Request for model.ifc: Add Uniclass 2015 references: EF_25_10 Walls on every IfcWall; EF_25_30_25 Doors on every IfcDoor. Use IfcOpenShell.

First a look at what the model holds.

```python
import ifcopenshell

model = ifcopenshell.open("model.ifc")
print(model.schema)
print("classifications:", [c.Name for c in model.by_type("IfcClassification")])
for ifc_class in ("IfcDoor", "IfcRoof", "IfcStair", "IfcWall", "IfcWindow"):
    print(ifc_class, len(model.by_type(ifc_class)))
```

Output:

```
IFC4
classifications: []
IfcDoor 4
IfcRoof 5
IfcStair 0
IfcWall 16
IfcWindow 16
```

```python
import ifcopenshell
import ifcopenshell.api.classification

model = ifcopenshell.open("model.ifc")

system = ifcopenshell.api.classification.add_classification(model, classification="Uniclass 2015")

codes = {
    "IfcWall": ("EF_25_10", "Walls"),
    "IfcDoor": ("EF_25_30_25", "Doors"),
}
for ifc_class, (code, name) in codes.items():
    products = model.by_type(ifc_class)
    ifcopenshell.api.classification.add_reference(
        model, products=products, classification=system, identification=code, name=name
    )
    print(code, len(products))

model.write("model-out.ifc")
```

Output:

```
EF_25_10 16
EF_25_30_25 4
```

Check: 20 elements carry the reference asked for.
